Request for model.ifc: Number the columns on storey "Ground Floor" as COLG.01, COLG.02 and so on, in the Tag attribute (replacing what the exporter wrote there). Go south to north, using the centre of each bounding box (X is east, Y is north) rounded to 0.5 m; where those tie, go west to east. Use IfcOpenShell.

First a look at what the model holds.

```python
import ifcopenshell
import ifcopenshell.util.element
import ifcopenshell.util.placement

model = ifcopenshell.open("model.ifc")
print(model.schema)
storey = next(s for s in model.by_type("IfcBuildingStorey") if s.Name == "Ground Floor")
columns = [e for e in ifcopenshell.util.element.get_decomposition(storey) if e.is_a("IfcColumn")]
for e in sorted(columns, key=lambda e: e.id()):
    origin = ifcopenshell.util.placement.get_local_placement(e.ObjectPlacement)[:3, 3]
    print(e.id(), e.Tag, e.Name, origin.round(2) + 0.0, sep=" | ")
```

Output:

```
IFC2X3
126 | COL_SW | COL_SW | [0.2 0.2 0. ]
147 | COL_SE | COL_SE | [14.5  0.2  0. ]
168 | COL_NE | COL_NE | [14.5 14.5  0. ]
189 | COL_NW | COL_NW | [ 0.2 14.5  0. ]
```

```python
import ifcopenshell
import ifcopenshell.geom
import ifcopenshell.util.element
import ifcopenshell.util.shape

model = ifcopenshell.open("model.ifc")
settings = ifcopenshell.geom.settings()
settings.set("use-world-coords", True)


def centre(element):
    shape = ifcopenshell.geom.create_shape(settings, element)
    return ifcopenshell.util.shape.get_bbox_centroid(shape.geometry)


storey = next(s for s in model.by_type("IfcBuildingStorey") if s.Name == "Ground Floor")
columns = [e for e in ifcopenshell.util.element.get_decomposition(storey) if e.is_a("IfcColumn")]

# Insertion points can sit at a corner or the storey origin, so sort by the geometry (in metres).
centres = {e: centre(e) for e in columns}
columns.sort(key=lambda e: (round(centres[e][1] / 0.5), centres[e][0]))

for i, e in enumerate(columns, start=1):
    number = f"COLG.{i:02d}"
    e.Tag = number
    print(e.id(), number)

model.write("model-out.ifc")
```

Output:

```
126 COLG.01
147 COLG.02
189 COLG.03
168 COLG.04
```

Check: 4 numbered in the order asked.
